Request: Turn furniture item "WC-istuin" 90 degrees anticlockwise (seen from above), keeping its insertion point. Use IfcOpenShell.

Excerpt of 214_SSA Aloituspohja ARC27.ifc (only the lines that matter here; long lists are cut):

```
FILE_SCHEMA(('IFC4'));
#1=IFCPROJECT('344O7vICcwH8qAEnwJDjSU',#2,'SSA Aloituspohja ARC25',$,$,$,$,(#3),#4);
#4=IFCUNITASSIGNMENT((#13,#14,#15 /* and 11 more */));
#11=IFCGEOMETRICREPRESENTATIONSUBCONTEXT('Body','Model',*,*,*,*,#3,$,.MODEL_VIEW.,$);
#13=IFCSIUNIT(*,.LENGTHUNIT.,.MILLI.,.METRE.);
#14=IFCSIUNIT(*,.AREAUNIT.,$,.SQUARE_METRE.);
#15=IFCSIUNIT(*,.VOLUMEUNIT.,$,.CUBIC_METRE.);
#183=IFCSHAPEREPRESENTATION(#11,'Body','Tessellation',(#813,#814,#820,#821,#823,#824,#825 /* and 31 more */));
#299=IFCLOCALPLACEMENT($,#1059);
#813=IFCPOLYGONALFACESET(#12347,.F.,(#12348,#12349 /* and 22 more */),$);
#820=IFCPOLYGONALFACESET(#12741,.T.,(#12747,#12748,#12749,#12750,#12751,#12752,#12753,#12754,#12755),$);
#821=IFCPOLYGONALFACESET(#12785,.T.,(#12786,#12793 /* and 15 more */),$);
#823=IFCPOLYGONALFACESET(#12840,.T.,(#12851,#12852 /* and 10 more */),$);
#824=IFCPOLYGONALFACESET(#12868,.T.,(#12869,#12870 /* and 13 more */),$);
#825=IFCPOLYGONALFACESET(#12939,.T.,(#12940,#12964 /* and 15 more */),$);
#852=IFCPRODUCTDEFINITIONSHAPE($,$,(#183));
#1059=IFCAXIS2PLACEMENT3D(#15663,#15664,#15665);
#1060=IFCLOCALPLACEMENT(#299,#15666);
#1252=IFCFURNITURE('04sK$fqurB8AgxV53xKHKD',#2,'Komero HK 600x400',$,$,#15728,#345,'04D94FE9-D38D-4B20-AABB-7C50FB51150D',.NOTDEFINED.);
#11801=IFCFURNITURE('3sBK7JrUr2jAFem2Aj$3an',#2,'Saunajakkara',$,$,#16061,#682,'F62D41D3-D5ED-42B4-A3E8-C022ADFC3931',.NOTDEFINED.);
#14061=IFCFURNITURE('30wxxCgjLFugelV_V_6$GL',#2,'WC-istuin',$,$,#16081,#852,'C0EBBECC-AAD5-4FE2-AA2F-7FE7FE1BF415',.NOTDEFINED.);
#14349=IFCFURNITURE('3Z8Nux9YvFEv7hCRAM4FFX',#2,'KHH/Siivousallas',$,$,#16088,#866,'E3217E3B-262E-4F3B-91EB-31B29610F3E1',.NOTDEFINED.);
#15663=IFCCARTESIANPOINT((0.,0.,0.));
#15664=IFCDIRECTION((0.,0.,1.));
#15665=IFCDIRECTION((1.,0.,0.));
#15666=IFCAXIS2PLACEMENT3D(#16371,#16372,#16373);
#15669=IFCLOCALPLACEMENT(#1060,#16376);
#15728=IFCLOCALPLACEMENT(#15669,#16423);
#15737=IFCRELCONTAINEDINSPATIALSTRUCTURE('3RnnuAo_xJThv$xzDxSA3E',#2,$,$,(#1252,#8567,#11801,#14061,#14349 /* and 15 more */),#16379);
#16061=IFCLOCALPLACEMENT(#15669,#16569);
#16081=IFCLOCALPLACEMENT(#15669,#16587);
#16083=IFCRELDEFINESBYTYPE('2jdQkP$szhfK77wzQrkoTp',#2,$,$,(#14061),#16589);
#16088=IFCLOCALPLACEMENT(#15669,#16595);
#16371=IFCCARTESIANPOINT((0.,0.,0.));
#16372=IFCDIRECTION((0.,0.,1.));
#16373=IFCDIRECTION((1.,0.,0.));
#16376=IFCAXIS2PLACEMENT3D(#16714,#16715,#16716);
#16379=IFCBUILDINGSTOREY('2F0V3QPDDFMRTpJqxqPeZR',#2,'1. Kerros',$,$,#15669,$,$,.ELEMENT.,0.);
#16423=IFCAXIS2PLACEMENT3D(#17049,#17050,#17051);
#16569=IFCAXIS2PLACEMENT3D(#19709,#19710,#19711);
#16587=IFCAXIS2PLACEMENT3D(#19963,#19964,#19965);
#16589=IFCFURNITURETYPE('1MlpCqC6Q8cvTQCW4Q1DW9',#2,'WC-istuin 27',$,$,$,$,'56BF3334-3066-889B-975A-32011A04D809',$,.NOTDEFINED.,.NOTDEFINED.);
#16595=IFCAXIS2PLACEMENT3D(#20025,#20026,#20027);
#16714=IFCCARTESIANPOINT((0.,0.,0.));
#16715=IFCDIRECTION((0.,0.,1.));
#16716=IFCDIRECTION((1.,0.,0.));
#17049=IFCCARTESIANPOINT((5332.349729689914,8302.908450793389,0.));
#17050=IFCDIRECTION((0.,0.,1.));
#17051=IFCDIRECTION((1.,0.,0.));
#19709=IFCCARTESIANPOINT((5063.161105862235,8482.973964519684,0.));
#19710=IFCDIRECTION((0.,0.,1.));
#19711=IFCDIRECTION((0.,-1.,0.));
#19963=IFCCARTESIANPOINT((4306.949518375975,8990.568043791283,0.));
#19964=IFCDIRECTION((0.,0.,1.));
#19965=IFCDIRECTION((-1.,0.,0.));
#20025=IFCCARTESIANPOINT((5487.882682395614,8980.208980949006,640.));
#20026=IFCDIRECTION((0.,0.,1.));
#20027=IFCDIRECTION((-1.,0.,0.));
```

```python
import ifcopenshell
import ifcopenshell.api.geometry
import ifcopenshell.util.placement

model = ifcopenshell.open("214_SSA Aloituspohja ARC27.ifc")

item = model.by_id(14061)
matrix = ifcopenshell.util.placement.get_local_placement(item.ObjectPlacement)
matrix = matrix @ ifcopenshell.util.placement.rotation(90, "Z")
ifcopenshell.api.geometry.edit_object_placement(model, product=item, matrix=matrix, is_si=False)

print(ifcopenshell.util.placement.get_local_placement(item.ObjectPlacement).round(3) + 0.0)

model.write("214_SSA Aloituspohja ARC27_v2.ifc")
```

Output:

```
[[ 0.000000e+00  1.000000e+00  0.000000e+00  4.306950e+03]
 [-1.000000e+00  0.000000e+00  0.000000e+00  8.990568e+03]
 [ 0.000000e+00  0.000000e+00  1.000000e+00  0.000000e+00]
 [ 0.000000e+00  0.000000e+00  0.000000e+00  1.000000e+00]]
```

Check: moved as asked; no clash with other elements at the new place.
